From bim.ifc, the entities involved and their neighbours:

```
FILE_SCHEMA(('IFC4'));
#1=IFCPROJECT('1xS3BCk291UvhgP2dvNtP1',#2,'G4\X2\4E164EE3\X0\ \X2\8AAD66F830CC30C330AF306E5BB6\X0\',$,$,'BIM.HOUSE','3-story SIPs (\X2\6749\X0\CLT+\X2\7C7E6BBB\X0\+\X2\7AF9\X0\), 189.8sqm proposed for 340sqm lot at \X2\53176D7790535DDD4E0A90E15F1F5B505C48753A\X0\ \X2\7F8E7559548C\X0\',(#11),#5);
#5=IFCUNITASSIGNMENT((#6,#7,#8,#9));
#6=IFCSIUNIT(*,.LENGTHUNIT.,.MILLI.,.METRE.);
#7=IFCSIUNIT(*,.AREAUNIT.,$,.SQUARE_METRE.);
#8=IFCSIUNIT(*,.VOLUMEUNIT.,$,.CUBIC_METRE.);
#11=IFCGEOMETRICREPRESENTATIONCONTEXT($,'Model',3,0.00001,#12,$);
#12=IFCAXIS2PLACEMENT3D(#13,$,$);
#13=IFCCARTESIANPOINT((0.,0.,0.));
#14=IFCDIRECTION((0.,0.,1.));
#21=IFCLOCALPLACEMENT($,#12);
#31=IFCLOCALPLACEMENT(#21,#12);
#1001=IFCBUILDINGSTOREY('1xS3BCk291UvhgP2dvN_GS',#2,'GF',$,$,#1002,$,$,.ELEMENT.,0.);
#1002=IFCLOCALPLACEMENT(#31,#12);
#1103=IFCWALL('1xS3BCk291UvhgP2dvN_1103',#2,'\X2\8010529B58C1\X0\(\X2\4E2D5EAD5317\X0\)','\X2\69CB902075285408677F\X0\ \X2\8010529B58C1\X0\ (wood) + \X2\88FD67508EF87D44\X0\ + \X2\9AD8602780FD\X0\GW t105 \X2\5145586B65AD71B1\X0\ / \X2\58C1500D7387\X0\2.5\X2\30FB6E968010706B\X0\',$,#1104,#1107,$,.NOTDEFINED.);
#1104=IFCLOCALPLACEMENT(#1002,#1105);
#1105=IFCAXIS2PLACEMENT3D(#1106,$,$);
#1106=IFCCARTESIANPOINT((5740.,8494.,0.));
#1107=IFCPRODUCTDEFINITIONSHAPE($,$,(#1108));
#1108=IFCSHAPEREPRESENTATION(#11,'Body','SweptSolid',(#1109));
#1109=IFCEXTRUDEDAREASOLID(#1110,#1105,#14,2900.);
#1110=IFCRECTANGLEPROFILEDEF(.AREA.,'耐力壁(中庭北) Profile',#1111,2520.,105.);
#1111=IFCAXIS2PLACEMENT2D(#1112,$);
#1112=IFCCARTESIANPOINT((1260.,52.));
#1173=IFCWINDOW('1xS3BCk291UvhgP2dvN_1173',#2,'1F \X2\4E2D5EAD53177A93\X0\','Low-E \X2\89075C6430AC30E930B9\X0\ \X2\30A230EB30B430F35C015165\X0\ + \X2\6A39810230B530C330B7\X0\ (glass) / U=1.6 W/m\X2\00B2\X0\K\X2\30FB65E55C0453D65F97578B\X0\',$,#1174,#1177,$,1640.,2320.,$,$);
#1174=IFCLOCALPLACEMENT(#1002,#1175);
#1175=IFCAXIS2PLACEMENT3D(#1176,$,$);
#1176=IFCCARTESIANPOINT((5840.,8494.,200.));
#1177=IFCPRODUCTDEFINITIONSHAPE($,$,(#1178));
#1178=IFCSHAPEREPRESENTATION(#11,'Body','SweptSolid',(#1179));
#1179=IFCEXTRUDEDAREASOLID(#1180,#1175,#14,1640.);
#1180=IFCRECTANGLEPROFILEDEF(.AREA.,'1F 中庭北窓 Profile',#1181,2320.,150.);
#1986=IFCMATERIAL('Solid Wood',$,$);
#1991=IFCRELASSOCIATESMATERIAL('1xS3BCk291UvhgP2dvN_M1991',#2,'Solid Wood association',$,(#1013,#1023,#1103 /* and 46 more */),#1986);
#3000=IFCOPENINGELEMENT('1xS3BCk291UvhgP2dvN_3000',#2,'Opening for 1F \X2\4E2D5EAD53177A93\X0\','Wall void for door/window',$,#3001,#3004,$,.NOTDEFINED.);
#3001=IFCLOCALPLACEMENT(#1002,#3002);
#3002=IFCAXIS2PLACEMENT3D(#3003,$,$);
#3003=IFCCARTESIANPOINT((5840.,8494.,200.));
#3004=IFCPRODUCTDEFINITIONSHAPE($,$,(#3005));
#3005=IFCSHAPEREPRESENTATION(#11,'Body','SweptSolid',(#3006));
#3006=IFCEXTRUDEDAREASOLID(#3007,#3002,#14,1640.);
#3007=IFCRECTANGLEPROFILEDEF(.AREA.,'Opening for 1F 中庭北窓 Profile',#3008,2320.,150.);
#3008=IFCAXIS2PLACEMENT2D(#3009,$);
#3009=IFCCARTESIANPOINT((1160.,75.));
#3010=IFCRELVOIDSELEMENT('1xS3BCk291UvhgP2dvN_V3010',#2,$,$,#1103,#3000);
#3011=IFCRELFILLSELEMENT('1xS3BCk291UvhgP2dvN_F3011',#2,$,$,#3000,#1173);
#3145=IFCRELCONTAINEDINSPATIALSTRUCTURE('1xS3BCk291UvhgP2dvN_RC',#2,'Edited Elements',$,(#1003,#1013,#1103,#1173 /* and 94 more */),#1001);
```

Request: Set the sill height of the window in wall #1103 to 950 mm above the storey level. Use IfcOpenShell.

```python
import numpy as np
import ifcopenshell
import ifcopenshell.api.geometry
import ifcopenshell.geom
import ifcopenshell.util.element
import ifcopenshell.util.placement
import ifcopenshell.util.shape
import ifcopenshell.util.unit

model = ifcopenshell.open("bim.ifc")
unit_scale = ifcopenshell.util.unit.calculate_unit_scale(model)

window = model.by_guid("1xS3BCk291UvhgP2dvN_1173")
opening = window.FillsVoids[0].RelatingOpeningElement
storey = ifcopenshell.util.element.get_container(window, ifc_class="IfcBuildingStorey")
level = ifcopenshell.util.placement.get_local_placement(storey.ObjectPlacement)[2, 3]

# The opening's origin need not be at the sill, so measure its lowest point.
shape = ifcopenshell.geom.create_shape(ifcopenshell.geom.settings(), opening)
bottom = ifcopenshell.util.shape.get_shape_bottom_elevation(shape, shape.geometry) / unit_scale
dz = level + 0.95 / unit_scale - bottom

shift = np.array([0.0, 0.0, dz])
# The window is not placed relative to its opening, so move both.
for product in (opening, window):
    matrix = ifcopenshell.util.placement.get_local_placement(product.ObjectPlacement)
    matrix[:3, 3] += shift
    ifcopenshell.api.geometry.edit_object_placement(model, product=product, matrix=matrix, is_si=False)

print(f"moved by {dz * unit_scale:+.3f} m")

model.write("bim_v2.ifc")
```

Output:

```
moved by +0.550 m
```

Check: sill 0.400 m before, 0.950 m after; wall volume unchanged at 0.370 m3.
